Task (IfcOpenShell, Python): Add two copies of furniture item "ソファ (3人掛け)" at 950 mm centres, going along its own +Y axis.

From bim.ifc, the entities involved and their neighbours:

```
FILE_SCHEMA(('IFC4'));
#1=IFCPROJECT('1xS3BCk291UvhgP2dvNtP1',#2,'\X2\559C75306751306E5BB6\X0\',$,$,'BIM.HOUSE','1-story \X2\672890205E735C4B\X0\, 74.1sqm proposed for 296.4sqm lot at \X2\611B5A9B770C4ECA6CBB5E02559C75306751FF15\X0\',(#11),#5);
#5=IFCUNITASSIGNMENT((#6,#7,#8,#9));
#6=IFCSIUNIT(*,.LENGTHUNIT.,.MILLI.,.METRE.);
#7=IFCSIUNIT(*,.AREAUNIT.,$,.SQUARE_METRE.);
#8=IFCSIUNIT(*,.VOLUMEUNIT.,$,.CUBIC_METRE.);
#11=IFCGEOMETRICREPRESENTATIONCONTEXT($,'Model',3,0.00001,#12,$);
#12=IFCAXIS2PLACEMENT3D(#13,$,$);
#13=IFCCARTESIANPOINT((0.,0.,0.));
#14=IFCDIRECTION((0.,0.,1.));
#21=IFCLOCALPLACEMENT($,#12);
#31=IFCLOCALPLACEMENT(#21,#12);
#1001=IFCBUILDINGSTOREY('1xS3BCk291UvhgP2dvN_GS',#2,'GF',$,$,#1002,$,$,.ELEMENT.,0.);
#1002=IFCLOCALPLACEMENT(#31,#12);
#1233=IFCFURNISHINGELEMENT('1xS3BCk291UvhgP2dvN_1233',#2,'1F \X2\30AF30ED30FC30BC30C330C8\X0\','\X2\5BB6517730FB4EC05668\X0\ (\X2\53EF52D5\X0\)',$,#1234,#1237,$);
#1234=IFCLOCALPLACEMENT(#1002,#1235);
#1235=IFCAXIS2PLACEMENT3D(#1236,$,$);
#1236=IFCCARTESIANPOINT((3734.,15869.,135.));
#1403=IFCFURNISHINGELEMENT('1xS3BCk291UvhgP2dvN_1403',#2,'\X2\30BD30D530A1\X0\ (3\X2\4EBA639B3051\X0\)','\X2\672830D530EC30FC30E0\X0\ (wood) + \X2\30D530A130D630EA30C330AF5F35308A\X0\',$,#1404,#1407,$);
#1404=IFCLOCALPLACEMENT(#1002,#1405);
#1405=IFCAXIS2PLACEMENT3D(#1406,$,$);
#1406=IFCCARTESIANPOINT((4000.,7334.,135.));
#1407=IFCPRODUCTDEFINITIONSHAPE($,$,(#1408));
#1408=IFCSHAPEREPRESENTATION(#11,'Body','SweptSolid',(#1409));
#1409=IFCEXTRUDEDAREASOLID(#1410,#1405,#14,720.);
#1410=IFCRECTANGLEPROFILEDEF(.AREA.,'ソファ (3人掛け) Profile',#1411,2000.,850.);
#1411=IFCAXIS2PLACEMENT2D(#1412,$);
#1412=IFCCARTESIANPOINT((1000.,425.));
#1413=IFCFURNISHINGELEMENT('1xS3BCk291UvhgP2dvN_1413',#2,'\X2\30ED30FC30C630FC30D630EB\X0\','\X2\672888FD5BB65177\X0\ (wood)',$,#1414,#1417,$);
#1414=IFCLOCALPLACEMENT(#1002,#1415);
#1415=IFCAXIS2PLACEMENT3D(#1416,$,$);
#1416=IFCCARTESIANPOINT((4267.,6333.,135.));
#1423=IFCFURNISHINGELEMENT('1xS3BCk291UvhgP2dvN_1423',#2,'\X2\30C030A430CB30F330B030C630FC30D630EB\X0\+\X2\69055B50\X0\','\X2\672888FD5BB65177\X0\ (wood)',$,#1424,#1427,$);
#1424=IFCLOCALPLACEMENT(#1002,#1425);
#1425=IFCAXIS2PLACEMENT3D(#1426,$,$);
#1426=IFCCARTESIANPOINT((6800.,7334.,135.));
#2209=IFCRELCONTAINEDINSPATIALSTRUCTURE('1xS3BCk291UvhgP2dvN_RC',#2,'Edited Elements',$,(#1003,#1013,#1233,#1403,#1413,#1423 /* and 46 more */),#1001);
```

```python
import ifcopenshell
import ifcopenshell.api.geometry
import ifcopenshell.api.root
import ifcopenshell.util.element
import ifcopenshell.util.placement

model = ifcopenshell.open("bim.ifc")


def reuse_history(source, copy):
    """copy_class also copies each property set's owner history, people and application; keep the originals."""
    for rel in copy.IsDefinedBy:
        if rel.is_a("IfcRelDefinesByProperties") and (history := rel.RelatingPropertyDefinition.OwnerHistory):
            rel.RelatingPropertyDefinition.OwnerHistory = source.OwnerHistory
            ifcopenshell.util.element.remove_deep2(model, history)


source = model.by_guid("1xS3BCk291UvhgP2dvN_1403")
base = ifcopenshell.util.placement.get_local_placement(source.ObjectPlacement)
step = base[:3, 1] * 950.0

for i in range(1, 3):
    copy = ifcopenshell.api.root.copy_class(model, product=source)
    copy.Representation = ifcopenshell.util.element.copy_deep(
        model, source.Representation, exclude=["IfcGeometricRepresentationContext", "IfcRepresentationMap"]
    )
    reuse_history(source, copy)
    matrix = base.copy()
    matrix[:3, 3] += i * step
    print("added at", matrix[:3, 3].round(3) + 0.0)
    ifcopenshell.api.geometry.edit_object_placement(model, product=copy, matrix=matrix, is_si=False)

model.write("bim_rev.ifc")
```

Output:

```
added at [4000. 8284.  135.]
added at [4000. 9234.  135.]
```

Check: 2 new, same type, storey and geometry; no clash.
